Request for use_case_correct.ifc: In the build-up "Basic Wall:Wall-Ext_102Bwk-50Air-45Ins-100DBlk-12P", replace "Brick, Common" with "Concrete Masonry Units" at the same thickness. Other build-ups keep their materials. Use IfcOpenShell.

First a look at what the model holds.

```python
import ifcopenshell
import ifcopenshell.util.element

model = ifcopenshell.open("use_case_correct.ifc")
print(model.schema)
for layer_set in model.by_type("IfcMaterialLayerSet"):
    if layer_set.LayerSetName == "Basic Wall:Wall-Ext_102Bwk-50Air-45Ins-100DBlk-12P":
        for layer in layer_set.MaterialLayers:
            print(layer.id(), layer.Material and layer.Material.Name, layer.LayerThickness, sep=" | ")
        print(len(ifcopenshell.util.element.get_elements_by_material(model, layer_set)), "elements and types use it")
print(sorted(m.Name for m in model.by_type("IfcMaterial") if m.Name)[:60])
```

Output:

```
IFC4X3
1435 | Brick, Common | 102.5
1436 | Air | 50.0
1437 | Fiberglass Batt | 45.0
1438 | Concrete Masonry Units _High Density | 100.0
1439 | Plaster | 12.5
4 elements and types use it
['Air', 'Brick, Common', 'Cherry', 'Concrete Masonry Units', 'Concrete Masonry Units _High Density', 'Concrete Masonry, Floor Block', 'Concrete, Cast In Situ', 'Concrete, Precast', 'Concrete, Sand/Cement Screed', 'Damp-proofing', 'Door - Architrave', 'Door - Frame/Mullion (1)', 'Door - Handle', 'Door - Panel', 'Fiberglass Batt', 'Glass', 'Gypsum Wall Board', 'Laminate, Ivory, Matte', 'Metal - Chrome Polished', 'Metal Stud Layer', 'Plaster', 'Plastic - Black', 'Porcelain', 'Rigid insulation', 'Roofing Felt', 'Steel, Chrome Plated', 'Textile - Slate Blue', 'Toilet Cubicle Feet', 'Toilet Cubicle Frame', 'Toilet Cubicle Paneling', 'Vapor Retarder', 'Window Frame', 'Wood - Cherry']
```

```python
import ifcopenshell
import ifcopenshell.api.material

model = ifcopenshell.open("use_case_correct.ifc")

layer_set = next(s for s in model.by_type("IfcMaterialLayerSet") if s.LayerSetName == "Basic Wall:Wall-Ext_102Bwk-50Air-45Ins-100DBlk-12P")
layer = next(l for l in layer_set.MaterialLayers if l.Material and l.Material.Name == "Brick, Common")
material = next(m for m in model.by_type("IfcMaterial") if m.Name == "Concrete Masonry Units")

# Point this one layer at the other material; renaming the old one would change it everywhere.
ifcopenshell.api.material.edit_layer(model, layer=layer, attributes={"Name": material.Name}, material=material)

print([l.Material.Name if l.Material else None for l in layer_set.MaterialLayers])

model.write("use_case_correct-out.ifc")
```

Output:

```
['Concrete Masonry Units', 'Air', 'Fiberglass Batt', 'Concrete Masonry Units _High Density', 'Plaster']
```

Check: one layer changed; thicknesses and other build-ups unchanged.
